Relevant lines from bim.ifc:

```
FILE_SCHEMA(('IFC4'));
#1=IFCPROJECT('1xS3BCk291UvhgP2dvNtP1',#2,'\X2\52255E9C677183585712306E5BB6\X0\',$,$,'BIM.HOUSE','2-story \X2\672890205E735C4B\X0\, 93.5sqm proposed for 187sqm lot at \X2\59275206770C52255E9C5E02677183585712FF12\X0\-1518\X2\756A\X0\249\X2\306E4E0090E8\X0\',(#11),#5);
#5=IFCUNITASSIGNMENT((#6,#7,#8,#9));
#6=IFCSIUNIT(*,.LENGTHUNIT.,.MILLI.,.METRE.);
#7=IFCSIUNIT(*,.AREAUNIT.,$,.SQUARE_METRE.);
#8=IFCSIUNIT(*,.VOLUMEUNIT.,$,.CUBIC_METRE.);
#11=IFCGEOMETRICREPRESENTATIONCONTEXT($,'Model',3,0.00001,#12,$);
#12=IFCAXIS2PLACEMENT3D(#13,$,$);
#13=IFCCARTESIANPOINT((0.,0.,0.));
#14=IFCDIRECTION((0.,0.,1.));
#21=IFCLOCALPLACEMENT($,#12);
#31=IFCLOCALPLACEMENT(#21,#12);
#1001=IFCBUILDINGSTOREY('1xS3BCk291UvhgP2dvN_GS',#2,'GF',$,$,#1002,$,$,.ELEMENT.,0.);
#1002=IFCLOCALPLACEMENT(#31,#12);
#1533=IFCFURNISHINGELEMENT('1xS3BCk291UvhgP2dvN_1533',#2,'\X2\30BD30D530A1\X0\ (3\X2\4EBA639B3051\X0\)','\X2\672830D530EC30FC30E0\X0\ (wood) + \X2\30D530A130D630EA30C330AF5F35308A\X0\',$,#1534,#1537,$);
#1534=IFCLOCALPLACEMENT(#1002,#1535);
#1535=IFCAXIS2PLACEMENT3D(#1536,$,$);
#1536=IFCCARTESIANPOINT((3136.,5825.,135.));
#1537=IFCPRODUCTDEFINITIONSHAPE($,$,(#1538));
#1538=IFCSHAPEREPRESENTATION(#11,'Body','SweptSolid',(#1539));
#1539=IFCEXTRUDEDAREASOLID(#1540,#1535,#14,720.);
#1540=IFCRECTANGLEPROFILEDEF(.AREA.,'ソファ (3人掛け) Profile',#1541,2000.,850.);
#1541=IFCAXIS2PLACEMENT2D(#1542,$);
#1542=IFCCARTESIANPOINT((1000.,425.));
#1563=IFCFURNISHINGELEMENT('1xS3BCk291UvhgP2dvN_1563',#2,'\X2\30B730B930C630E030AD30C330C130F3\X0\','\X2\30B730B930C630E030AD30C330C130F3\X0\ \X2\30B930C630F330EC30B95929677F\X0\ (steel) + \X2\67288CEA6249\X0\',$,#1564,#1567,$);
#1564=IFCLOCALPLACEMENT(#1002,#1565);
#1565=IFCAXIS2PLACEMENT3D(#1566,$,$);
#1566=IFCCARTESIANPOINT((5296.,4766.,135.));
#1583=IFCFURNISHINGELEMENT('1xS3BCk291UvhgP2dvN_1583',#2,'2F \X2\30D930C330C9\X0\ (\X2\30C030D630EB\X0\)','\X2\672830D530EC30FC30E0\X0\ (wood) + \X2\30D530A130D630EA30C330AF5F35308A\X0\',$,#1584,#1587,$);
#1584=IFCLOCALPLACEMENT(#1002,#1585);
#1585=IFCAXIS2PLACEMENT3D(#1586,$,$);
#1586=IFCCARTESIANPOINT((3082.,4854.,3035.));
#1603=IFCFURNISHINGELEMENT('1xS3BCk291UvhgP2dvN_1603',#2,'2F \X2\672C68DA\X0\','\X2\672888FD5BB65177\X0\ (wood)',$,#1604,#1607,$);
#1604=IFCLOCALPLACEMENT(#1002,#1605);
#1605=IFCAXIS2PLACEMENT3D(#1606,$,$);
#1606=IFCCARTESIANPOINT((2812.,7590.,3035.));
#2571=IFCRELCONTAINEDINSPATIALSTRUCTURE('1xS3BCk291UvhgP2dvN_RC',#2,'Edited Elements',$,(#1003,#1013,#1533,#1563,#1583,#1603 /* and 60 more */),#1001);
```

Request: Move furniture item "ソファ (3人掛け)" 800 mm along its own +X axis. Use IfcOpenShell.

```python
import ifcopenshell
import ifcopenshell.api.geometry
import ifcopenshell.util.placement
import ifcopenshell.util.unit

model = ifcopenshell.open("bim.ifc")
unit_scale = ifcopenshell.util.unit.calculate_unit_scale(model)

item = model.by_guid("1xS3BCk291UvhgP2dvN_1533")
matrix = ifcopenshell.util.placement.get_local_placement(item.ObjectPlacement)
matrix[:3, 3] += matrix[:3, 0] * 0.8 / unit_scale
ifcopenshell.api.geometry.edit_object_placement(model, product=item, matrix=matrix, is_si=False)

print(ifcopenshell.util.placement.get_local_placement(item.ObjectPlacement).round(3) + 0.0)

model.write("bim_edited.ifc")
```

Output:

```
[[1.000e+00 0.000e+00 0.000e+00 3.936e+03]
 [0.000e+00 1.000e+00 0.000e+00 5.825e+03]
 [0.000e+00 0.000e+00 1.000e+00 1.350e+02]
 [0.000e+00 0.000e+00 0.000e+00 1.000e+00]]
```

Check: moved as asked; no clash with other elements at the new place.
